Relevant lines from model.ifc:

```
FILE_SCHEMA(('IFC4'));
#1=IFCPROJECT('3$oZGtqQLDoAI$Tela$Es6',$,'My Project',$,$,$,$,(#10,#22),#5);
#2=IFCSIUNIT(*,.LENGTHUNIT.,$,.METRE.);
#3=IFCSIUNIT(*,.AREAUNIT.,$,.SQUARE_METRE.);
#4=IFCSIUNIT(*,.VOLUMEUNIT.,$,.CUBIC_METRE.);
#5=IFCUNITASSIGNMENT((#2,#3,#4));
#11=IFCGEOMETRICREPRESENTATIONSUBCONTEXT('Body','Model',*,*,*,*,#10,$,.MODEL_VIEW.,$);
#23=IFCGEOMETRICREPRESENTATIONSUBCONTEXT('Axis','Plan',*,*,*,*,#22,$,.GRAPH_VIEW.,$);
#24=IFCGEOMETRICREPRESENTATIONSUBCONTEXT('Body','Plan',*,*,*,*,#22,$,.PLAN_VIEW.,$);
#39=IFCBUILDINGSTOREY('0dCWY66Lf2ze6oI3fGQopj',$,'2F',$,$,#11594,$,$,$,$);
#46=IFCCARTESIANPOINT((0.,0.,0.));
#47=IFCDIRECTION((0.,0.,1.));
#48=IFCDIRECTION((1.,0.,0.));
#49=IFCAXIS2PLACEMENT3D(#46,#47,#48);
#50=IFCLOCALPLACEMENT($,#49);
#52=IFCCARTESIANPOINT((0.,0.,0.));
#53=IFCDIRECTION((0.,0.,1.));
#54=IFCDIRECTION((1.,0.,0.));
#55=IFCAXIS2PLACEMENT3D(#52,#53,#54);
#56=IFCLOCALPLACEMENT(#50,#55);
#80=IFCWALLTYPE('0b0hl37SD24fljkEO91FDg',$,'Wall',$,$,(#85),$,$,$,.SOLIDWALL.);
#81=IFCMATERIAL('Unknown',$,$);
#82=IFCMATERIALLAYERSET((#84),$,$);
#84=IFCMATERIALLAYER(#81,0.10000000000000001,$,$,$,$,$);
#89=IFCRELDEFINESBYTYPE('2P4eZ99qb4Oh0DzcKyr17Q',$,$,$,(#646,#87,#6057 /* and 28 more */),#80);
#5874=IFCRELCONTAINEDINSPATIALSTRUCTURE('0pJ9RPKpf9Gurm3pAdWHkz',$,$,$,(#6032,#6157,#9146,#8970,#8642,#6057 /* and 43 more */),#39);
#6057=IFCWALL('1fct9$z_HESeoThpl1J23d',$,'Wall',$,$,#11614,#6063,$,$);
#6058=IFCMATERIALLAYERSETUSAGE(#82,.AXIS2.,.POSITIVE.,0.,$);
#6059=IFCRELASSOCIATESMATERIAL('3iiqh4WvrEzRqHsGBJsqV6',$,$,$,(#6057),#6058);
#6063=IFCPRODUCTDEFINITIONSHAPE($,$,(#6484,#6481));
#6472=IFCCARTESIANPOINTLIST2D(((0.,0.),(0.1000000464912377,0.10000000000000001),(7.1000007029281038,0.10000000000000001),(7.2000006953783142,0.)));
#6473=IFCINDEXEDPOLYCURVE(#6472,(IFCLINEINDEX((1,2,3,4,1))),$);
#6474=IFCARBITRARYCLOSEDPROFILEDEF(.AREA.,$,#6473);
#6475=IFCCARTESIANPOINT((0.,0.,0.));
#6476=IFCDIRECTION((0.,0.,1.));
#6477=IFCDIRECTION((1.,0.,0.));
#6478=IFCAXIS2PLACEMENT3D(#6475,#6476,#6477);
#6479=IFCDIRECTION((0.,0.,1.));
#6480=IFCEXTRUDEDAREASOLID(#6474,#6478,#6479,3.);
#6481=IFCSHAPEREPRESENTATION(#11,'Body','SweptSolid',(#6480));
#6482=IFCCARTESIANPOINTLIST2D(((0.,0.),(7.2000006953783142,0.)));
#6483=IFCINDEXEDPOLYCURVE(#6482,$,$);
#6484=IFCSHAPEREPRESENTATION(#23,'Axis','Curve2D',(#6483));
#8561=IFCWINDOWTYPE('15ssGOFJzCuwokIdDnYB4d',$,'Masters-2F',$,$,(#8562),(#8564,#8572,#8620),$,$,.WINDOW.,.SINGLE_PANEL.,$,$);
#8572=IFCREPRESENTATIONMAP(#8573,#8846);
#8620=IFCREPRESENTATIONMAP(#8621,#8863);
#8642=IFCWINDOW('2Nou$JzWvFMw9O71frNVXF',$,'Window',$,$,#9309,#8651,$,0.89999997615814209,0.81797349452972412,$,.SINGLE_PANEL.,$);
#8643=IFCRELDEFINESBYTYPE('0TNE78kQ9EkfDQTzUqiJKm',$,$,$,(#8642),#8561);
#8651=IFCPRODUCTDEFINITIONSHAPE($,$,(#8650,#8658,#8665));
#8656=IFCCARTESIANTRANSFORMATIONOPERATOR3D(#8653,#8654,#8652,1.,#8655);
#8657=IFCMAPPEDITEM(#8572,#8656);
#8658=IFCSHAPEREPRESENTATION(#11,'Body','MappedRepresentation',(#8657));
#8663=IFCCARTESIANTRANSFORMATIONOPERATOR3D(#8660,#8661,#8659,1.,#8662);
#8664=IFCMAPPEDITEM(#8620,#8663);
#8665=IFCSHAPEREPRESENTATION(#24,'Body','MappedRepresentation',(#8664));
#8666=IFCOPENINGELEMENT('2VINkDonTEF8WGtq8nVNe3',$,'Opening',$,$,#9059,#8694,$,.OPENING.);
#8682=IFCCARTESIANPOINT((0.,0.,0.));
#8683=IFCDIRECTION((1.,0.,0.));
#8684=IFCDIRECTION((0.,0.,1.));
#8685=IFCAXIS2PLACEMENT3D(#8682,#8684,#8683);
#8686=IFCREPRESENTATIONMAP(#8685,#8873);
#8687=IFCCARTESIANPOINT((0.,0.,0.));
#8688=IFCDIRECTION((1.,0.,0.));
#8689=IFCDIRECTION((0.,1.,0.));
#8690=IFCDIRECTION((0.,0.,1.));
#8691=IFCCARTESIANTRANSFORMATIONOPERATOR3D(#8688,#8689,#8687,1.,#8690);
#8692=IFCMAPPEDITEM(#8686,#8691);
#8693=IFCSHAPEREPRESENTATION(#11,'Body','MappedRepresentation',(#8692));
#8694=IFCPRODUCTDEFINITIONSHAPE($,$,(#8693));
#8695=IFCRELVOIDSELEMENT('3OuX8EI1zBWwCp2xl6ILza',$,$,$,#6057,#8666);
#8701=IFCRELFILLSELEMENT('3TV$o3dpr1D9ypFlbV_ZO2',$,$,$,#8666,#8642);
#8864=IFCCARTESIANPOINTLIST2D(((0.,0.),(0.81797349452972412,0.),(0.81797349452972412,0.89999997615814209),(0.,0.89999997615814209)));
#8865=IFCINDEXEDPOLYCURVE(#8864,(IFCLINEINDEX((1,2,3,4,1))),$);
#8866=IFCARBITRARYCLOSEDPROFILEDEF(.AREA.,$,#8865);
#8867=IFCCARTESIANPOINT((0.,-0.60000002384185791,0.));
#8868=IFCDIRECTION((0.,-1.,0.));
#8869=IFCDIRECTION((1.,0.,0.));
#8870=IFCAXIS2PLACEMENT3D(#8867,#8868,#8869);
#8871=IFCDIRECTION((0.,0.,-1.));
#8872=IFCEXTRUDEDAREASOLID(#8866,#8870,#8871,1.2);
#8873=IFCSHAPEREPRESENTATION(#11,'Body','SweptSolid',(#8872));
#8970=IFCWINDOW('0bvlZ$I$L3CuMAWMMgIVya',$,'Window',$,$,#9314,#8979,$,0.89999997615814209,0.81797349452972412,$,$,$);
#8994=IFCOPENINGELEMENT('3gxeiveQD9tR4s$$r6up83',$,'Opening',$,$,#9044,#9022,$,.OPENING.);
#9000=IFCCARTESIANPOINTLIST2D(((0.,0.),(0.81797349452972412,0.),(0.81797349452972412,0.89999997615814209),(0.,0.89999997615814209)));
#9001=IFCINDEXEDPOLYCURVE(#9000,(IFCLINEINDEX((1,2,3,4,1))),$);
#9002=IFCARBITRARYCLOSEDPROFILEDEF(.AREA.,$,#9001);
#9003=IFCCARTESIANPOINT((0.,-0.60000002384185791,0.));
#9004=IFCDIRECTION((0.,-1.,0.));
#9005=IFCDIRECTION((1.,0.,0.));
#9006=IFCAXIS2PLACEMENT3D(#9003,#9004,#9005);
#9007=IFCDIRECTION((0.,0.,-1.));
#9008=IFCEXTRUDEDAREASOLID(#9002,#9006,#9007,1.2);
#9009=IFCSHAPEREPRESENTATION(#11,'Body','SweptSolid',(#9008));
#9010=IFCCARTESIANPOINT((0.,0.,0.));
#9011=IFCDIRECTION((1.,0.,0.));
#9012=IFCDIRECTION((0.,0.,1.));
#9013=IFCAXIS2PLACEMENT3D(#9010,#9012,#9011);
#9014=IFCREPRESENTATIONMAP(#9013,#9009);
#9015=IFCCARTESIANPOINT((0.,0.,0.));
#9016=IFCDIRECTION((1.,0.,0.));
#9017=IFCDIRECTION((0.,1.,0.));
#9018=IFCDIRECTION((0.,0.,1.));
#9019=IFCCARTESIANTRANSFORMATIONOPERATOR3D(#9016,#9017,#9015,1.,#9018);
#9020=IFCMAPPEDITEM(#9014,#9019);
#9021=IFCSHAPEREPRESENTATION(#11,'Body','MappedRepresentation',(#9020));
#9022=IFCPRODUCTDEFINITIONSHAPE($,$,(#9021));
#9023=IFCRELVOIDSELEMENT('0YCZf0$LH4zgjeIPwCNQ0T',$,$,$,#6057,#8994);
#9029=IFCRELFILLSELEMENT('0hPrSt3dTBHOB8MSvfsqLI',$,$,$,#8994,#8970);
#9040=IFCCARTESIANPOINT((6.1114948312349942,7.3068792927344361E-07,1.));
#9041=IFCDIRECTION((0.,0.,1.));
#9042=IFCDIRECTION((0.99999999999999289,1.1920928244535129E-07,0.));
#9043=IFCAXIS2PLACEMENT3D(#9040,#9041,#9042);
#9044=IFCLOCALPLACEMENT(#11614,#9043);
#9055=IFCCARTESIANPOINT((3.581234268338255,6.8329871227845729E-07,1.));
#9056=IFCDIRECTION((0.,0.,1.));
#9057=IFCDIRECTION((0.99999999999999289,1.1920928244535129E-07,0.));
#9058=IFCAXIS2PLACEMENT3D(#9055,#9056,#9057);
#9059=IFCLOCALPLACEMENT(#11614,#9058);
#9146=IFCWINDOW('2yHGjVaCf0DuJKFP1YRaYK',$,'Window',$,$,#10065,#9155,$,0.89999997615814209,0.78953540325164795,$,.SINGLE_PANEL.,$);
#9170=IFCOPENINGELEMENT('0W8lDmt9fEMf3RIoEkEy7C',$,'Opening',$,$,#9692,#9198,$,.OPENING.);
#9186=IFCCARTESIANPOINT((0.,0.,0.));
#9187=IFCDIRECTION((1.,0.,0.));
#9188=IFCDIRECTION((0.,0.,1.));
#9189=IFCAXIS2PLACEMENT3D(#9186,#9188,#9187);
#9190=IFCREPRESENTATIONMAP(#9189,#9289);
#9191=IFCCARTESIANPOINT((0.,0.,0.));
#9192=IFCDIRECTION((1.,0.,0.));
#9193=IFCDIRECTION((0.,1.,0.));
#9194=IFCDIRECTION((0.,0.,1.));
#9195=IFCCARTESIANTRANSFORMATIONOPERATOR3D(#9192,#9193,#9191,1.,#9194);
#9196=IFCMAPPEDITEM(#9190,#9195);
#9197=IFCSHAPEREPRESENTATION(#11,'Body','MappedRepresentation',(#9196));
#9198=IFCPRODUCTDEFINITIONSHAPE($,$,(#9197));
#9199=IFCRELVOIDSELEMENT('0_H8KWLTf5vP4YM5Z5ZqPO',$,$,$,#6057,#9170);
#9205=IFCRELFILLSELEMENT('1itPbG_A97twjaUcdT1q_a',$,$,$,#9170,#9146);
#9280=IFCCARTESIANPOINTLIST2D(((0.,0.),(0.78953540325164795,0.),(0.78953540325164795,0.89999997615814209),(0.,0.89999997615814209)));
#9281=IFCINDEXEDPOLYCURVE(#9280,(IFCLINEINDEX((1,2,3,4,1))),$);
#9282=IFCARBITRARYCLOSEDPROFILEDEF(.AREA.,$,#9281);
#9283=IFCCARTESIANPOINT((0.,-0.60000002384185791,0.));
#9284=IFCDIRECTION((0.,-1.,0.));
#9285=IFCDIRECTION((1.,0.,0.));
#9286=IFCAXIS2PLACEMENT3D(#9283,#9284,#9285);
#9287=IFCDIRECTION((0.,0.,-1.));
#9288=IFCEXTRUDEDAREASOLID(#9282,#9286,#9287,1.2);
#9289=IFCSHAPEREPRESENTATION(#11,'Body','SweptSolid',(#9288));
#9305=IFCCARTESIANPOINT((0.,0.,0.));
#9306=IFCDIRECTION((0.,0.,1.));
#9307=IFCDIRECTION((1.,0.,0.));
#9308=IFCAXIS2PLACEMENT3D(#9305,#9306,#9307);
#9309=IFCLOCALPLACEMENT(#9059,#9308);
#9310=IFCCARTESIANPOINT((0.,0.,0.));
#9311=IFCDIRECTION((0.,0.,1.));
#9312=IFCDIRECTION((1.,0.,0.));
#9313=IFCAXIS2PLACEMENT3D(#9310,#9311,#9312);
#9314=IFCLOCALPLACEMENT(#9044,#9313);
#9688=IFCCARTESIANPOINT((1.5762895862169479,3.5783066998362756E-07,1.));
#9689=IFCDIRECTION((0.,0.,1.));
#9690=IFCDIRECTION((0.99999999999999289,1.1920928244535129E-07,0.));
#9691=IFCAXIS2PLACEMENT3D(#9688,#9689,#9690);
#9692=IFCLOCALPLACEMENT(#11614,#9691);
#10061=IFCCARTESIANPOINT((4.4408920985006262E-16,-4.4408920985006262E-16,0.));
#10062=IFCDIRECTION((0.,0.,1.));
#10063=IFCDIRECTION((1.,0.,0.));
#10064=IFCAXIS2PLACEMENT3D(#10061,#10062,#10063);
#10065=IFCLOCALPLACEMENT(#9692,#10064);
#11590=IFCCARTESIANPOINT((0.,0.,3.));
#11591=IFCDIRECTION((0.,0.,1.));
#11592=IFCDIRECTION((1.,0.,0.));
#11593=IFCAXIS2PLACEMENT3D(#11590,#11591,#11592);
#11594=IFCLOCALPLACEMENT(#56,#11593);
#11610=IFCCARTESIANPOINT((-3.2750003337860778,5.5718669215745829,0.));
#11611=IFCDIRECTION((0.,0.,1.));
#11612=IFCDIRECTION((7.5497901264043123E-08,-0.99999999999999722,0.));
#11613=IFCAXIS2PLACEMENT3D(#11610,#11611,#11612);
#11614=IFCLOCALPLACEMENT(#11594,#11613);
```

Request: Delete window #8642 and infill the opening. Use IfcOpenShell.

```python
import ifcopenshell
import ifcopenshell.api.feature
import ifcopenshell.api.root
import ifcopenshell.geom
import ifcopenshell.util.shape

model = ifcopenshell.open("model.ifc")
settings = ifcopenshell.geom.settings()


def volume(element):
    """Net volume in cubic metres, openings subtracted."""
    shape = ifcopenshell.geom.create_shape(settings, element)
    return ifcopenshell.util.shape.get_volume(shape.geometry)


window = model.by_guid("2Nou$JzWvFMw9O71frNVXF")
opening = window.FillsVoids[0].RelatingOpeningElement
wall = opening.VoidsElements[0].RelatingBuildingElement
before = volume(wall)

ifcopenshell.api.root.remove_product(model, product=window)
ifcopenshell.api.feature.remove_feature(model, feature=opening)

after = volume(wall)

print(f"wall volume {before:.3f} -> {after:.3f} m3")

model.write("model_updated.ifc")
```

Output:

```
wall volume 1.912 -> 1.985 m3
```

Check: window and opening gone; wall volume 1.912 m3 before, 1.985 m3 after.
